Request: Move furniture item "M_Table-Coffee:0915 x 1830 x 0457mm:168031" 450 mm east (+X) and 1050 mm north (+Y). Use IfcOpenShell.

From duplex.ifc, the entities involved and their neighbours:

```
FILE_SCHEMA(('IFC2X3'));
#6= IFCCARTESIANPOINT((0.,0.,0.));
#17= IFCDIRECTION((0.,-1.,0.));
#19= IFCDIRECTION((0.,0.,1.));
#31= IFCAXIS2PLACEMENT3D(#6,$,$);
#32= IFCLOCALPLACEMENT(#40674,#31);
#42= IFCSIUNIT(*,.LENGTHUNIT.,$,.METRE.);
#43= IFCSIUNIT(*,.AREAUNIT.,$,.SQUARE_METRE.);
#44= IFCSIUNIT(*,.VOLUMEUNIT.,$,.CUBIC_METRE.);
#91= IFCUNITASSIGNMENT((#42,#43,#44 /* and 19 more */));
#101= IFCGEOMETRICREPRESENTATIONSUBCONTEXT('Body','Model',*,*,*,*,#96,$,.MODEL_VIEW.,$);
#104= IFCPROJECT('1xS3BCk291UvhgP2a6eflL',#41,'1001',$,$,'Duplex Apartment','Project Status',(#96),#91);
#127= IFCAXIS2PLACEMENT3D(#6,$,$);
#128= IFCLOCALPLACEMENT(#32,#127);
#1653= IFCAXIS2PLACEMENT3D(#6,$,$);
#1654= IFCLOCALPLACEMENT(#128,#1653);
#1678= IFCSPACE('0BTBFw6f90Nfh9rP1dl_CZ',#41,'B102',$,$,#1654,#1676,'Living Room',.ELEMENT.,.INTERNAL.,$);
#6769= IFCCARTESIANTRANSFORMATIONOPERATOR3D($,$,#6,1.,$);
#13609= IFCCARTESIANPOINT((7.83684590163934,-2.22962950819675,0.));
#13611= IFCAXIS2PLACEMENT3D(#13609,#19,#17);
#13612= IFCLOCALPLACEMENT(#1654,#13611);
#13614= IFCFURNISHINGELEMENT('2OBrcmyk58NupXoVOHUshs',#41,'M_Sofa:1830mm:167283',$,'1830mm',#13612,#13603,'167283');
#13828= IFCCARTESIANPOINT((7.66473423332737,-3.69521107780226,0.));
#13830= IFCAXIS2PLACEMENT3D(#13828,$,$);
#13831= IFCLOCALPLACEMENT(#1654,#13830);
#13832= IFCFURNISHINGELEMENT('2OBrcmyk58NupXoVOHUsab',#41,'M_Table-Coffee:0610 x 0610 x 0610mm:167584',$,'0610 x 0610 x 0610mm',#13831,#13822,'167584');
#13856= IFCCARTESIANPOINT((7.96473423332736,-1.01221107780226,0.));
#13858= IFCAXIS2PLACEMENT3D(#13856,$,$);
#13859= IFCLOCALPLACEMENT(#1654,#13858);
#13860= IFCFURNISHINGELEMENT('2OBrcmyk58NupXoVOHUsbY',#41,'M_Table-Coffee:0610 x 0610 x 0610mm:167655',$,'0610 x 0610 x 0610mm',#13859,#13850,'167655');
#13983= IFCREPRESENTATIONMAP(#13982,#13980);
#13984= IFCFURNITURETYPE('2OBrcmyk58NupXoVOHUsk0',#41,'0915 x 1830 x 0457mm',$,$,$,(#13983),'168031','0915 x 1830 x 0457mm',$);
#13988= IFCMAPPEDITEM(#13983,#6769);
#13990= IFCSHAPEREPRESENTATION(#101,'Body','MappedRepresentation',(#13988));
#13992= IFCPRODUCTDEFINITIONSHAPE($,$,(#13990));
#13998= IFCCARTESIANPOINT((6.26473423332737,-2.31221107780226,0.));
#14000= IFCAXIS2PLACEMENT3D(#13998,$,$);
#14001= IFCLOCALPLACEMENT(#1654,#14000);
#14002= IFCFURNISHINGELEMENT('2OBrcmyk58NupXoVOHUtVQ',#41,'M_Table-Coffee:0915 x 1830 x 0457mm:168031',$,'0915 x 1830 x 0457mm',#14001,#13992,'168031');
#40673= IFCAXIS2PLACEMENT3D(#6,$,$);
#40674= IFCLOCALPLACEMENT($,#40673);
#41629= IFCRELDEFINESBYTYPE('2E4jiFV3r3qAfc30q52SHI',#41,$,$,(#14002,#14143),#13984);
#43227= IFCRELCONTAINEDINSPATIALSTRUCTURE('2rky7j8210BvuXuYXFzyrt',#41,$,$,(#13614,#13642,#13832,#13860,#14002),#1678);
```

```python
import ifcopenshell
import ifcopenshell.api.geometry
import ifcopenshell.util.placement

model = ifcopenshell.open("duplex.ifc")

item = model.by_guid("2OBrcmyk58NupXoVOHUtVQ")
matrix = ifcopenshell.util.placement.get_local_placement(item.ObjectPlacement)
matrix[0, 3] += 0.45
matrix[1, 3] += 1.05
ifcopenshell.api.geometry.edit_object_placement(model, product=item, matrix=matrix, is_si=False)

print(ifcopenshell.util.placement.get_local_placement(item.ObjectPlacement).round(3) + 0.0)

model.write("duplex_edited.ifc")
```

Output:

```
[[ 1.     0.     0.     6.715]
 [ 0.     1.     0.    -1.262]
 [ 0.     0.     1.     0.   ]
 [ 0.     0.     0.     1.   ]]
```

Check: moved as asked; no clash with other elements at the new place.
